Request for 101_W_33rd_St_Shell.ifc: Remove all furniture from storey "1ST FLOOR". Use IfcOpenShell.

First a look at what the model holds.

```python
import ifcopenshell
import ifcopenshell.util.element

model = ifcopenshell.open("101_W_33rd_St_Shell.ifc")
print(model.schema)
storey = next(s for s in model.by_type("IfcBuildingStorey") if s.Name == "1ST FLOOR")
furniture = [e for e in ifcopenshell.util.element.get_decomposition(storey) if e.is_a("IfcFurnishingElement")]
seen = {}
for e in furniture:
    element_type = ifcopenshell.util.element.get_type(e)
    name = element_type.Name if element_type not in (None, e) else None
    seen[name] = seen.get(name, 0) + 1
for name, count in sorted(seen.items(), key=str):
    print(count, "x", name)
```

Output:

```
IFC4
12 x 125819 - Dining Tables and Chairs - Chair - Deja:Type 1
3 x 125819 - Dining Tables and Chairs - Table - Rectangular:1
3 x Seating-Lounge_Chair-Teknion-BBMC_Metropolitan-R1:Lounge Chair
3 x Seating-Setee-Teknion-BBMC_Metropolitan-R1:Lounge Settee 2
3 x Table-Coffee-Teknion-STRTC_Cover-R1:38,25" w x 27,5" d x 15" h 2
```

```python
import ifcopenshell
import ifcopenshell.api.root
import ifcopenshell.util.element

model = ifcopenshell.open("101_W_33rd_St_Shell.ifc")

storey = next(s for s in model.by_type("IfcBuildingStorey") if s.Name == "1ST FLOOR")
furniture = [e for e in ifcopenshell.util.element.get_decomposition(storey) if e.is_a("IfcFurnishingElement")]

for e in furniture:
    ifcopenshell.api.root.remove_product(model, product=e)
print(len(furniture), "removed")

model.write("101_W_33rd_St_Shell_updated.ifc")
```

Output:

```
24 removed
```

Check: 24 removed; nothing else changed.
